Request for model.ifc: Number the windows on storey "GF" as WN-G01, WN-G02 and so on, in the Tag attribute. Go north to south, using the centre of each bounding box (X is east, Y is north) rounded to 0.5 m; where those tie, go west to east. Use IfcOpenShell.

First a look at what the model holds.

```python
import ifcopenshell
import ifcopenshell.util.element
import ifcopenshell.util.placement

model = ifcopenshell.open("model.ifc")
print(model.schema)
storey = next(s for s in model.by_type("IfcBuildingStorey") if s.Name == "GF")
windows = [e for e in ifcopenshell.util.element.get_decomposition(storey) if e.is_a("IfcWindow")]
for e in sorted(windows, key=lambda e: e.id()):
    origin = ifcopenshell.util.placement.get_local_placement(e.ObjectPlacement)[:3, 3]
    print(e.id(), e.Tag, e.Name, origin.round(2) + 0.0, sep=" | ")
```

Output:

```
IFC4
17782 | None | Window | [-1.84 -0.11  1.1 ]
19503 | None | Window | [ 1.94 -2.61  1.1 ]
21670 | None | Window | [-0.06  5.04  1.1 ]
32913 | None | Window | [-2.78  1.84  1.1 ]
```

```python
import ifcopenshell
import ifcopenshell.geom
import ifcopenshell.util.element
import ifcopenshell.util.shape

model = ifcopenshell.open("model.ifc")
settings = ifcopenshell.geom.settings()
settings.set("use-world-coords", True)


def centre(element):
    shape = ifcopenshell.geom.create_shape(settings, element)
    return ifcopenshell.util.shape.get_bbox_centroid(shape.geometry)


storey = next(s for s in model.by_type("IfcBuildingStorey") if s.Name == "GF")
windows = [e for e in ifcopenshell.util.element.get_decomposition(storey) if e.is_a("IfcWindow")]

# Insertion points can sit at a corner or the storey origin, so sort by the geometry (in metres).
centres = {e: centre(e) for e in windows}
windows.sort(key=lambda e: (-round(centres[e][1] / 0.5), centres[e][0]))

for i, e in enumerate(windows, start=1):
    number = f"WN-G{i:02d}"
    e.Tag = number
    print(e.id(), number)

model.write("model_rev.ifc")
```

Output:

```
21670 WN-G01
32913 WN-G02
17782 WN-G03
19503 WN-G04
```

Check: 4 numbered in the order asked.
